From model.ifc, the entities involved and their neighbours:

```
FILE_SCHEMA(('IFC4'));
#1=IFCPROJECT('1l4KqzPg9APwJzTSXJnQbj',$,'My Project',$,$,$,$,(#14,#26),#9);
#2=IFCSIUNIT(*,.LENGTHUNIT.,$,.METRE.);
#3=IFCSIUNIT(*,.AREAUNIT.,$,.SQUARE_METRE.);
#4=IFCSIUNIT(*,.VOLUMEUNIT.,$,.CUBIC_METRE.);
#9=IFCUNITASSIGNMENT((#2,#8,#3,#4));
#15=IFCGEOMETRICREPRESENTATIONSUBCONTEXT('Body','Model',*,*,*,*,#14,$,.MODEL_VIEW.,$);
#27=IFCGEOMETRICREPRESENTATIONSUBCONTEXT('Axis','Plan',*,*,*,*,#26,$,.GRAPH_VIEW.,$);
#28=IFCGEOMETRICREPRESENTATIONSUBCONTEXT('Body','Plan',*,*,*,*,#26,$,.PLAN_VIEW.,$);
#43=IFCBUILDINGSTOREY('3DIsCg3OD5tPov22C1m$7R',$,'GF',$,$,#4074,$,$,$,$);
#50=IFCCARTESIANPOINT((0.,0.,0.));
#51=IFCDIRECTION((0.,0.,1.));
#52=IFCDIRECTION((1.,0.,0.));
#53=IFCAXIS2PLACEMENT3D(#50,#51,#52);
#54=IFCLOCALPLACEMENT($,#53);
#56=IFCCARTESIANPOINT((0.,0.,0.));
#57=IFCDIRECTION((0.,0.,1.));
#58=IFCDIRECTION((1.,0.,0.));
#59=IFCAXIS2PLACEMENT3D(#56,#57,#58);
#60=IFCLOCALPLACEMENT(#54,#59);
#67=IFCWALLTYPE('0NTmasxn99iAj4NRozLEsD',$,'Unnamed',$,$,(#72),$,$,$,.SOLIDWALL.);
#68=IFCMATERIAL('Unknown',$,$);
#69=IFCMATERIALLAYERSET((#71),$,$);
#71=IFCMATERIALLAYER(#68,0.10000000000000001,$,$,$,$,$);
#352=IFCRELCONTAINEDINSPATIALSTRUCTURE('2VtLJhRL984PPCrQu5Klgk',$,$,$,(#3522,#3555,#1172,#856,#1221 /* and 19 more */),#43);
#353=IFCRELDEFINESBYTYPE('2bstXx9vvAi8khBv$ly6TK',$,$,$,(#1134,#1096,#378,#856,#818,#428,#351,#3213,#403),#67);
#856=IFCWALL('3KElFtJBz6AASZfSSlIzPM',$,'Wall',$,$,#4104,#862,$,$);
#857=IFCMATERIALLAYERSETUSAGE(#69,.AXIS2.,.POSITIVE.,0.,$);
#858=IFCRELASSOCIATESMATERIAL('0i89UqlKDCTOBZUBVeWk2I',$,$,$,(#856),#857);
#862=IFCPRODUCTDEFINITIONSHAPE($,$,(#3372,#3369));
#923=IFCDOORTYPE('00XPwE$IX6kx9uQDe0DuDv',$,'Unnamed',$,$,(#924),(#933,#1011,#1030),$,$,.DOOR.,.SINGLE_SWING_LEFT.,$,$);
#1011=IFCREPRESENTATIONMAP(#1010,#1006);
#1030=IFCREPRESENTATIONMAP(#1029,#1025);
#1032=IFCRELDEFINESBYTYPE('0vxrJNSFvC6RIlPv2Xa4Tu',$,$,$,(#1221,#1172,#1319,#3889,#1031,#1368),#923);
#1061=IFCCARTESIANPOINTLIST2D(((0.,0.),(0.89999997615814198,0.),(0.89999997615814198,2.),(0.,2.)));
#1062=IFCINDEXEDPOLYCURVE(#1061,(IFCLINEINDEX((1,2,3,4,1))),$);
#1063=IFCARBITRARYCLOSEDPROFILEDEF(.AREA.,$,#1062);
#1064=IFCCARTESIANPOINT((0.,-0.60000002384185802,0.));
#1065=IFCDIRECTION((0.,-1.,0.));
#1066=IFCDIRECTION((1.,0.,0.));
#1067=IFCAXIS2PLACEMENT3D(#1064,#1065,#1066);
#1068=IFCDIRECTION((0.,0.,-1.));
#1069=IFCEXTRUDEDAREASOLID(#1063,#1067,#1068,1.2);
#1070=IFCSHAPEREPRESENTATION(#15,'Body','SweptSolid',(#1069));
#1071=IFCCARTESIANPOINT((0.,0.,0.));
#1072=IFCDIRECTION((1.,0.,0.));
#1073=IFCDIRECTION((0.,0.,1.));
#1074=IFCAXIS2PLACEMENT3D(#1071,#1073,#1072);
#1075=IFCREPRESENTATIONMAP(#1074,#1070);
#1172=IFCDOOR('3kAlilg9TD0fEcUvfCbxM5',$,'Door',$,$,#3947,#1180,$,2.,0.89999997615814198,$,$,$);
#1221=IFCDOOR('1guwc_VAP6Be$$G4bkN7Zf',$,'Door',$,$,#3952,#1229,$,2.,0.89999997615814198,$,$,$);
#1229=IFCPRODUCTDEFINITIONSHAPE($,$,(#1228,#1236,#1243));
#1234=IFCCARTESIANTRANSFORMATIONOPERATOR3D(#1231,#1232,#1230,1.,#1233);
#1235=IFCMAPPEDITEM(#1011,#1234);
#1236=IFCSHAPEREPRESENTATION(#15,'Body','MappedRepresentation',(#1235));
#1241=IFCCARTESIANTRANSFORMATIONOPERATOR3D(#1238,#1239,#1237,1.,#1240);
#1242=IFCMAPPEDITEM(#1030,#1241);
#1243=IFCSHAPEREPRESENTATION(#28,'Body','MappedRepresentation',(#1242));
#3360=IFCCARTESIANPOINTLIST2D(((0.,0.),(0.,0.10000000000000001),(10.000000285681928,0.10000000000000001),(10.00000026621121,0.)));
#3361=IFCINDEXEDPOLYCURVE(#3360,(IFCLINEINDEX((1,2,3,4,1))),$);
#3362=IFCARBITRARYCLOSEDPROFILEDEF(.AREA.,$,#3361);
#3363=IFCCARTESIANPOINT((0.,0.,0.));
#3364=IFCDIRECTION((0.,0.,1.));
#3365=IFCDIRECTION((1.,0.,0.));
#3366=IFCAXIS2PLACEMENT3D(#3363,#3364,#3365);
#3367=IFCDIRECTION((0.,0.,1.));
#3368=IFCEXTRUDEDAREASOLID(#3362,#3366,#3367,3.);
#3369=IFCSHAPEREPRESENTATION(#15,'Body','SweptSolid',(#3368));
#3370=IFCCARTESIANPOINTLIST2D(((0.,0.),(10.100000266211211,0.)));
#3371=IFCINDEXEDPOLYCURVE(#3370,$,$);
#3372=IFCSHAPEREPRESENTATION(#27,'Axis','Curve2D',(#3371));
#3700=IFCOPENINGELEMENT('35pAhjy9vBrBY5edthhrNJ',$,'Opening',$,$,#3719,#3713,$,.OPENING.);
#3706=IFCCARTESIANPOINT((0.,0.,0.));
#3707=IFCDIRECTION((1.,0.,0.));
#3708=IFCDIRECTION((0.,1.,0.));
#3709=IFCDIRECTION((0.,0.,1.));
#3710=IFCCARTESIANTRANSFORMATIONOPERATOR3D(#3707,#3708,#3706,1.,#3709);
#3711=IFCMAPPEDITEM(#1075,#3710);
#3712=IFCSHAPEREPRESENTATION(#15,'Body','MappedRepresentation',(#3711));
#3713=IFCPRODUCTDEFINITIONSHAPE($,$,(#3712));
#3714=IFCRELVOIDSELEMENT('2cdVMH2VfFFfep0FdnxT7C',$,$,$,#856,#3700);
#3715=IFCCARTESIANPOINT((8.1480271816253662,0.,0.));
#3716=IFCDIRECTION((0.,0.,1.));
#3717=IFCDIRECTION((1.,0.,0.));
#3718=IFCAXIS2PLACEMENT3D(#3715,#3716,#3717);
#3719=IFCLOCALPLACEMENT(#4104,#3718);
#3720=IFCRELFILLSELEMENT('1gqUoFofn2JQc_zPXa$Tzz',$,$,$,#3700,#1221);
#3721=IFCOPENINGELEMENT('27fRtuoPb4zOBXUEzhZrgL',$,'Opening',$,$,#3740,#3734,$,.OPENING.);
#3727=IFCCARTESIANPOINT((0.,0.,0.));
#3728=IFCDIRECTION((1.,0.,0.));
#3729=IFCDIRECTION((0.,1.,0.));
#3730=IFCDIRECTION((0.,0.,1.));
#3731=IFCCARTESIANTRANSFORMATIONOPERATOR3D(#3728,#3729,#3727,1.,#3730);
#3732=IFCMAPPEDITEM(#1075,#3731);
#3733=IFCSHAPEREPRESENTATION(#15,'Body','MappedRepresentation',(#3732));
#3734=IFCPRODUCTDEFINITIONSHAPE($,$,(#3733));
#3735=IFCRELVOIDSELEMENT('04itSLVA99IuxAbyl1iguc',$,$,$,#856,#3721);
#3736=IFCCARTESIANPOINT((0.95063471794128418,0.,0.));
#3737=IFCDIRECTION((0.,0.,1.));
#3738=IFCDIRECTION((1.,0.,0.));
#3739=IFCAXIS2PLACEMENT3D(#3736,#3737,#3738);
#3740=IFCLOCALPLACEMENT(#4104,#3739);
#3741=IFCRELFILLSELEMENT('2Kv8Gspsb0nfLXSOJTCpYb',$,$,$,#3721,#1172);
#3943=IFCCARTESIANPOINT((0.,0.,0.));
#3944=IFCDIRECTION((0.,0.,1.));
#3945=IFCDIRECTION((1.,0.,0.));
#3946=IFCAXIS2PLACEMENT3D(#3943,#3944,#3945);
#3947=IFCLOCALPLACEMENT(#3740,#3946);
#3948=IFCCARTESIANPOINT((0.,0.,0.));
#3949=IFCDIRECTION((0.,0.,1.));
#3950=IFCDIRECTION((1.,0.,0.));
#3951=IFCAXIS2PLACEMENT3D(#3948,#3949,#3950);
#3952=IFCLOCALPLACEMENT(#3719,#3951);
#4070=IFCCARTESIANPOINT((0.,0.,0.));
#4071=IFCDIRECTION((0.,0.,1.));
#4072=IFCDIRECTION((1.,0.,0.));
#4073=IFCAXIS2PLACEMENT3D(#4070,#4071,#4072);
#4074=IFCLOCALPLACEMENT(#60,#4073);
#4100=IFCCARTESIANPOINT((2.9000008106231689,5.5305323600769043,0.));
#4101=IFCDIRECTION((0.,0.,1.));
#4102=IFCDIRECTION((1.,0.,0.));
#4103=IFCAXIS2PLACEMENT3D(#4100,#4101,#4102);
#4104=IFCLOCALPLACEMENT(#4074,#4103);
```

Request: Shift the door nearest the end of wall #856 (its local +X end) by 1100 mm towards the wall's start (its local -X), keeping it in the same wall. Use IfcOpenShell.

```python
import ifcopenshell
import ifcopenshell.api.geometry
import ifcopenshell.util.placement
import ifcopenshell.util.unit

model = ifcopenshell.open("model.ifc")
unit_scale = ifcopenshell.util.unit.calculate_unit_scale(model)

door = model.by_guid("1guwc_VAP6Be$$G4bkN7Zf")
opening = door.FillsVoids[0].RelatingOpeningElement
wall = opening.VoidsElements[0].RelatingBuildingElement

wall_matrix = ifcopenshell.util.placement.get_local_placement(wall.ObjectPlacement)
shift = wall_matrix[:3, 0] * -1.1 / unit_scale
before = ifcopenshell.util.placement.get_local_placement(door.ObjectPlacement)[:3, 3].copy()

# The door is placed relative to its opening, so it follows when the opening moves.
matrix = ifcopenshell.util.placement.get_local_placement(opening.ObjectPlacement)
matrix[:3, 3] += shift
ifcopenshell.api.geometry.edit_object_placement(
    model, product=opening, matrix=matrix, is_si=False, should_transform_children=True
)

after = ifcopenshell.util.placement.get_local_placement(door.ObjectPlacement)[:3, 3]
print("door moved by", (after - before).round(3) + 0.0)

model.write("model_updated.ifc")
```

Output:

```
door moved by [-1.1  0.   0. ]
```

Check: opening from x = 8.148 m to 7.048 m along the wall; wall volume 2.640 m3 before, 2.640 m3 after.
